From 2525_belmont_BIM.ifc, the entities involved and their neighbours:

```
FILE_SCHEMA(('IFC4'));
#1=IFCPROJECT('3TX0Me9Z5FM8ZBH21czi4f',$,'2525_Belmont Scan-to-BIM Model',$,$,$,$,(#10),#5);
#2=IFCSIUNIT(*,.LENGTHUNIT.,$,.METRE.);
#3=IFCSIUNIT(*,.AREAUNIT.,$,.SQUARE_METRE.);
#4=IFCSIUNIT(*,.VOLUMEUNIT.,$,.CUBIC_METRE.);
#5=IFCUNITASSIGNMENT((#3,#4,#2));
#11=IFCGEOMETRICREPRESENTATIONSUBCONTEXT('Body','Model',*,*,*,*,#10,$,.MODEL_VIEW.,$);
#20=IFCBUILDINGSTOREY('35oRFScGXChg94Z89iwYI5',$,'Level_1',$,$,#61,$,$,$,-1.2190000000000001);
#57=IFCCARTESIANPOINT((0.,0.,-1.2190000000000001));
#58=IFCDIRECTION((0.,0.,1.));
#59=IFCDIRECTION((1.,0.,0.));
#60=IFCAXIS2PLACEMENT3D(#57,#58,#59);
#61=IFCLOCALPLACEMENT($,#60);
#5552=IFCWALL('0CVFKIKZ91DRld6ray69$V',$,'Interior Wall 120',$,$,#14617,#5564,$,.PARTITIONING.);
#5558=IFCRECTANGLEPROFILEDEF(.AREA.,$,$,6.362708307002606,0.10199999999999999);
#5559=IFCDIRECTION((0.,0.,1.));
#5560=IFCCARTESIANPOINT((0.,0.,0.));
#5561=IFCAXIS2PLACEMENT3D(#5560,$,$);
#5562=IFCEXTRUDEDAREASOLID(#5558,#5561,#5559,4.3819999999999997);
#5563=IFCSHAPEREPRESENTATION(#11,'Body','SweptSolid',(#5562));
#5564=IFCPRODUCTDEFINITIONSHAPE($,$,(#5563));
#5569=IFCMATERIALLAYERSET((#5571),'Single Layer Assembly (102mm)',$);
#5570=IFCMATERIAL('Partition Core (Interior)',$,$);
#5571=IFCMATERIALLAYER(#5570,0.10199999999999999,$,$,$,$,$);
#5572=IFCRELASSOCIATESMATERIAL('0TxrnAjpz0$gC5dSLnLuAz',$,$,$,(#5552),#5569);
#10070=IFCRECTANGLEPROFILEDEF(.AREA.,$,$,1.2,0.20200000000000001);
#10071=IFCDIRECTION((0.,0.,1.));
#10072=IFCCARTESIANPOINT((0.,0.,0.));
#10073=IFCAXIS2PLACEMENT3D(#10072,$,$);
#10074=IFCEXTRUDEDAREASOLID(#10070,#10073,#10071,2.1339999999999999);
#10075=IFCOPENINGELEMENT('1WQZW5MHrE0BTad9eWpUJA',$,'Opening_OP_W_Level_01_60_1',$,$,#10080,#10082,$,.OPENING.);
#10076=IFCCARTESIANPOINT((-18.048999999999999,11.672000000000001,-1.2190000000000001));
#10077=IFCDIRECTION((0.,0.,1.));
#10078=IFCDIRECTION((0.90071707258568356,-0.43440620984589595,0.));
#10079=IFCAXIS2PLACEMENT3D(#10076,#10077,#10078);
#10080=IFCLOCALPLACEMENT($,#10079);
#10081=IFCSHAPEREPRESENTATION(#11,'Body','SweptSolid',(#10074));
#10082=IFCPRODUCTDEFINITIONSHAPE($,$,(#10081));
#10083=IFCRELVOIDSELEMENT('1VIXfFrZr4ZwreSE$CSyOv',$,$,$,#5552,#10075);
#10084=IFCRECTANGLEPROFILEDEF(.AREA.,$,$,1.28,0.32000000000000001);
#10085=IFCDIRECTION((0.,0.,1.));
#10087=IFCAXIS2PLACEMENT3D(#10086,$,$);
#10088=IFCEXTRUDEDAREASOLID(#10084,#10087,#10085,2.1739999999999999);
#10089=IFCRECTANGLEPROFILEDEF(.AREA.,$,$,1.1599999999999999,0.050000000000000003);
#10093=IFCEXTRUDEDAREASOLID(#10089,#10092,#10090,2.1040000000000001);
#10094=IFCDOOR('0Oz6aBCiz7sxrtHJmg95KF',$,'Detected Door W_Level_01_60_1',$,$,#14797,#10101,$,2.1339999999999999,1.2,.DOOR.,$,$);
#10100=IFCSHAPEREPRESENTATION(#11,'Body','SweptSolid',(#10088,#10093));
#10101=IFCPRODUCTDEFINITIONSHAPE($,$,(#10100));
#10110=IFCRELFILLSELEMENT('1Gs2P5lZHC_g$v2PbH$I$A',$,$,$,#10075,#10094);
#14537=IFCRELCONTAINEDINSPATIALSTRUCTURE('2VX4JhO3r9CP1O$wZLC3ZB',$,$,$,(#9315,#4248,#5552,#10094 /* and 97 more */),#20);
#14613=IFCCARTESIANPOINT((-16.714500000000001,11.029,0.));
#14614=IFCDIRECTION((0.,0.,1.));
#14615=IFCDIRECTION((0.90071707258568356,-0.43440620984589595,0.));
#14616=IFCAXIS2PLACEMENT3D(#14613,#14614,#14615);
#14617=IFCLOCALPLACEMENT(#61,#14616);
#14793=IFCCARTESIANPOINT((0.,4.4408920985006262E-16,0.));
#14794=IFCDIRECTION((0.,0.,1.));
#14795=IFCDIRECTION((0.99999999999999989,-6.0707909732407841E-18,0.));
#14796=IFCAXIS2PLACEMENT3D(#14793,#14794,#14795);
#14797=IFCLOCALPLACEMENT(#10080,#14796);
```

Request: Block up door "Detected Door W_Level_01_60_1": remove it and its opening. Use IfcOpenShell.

```python
import ifcopenshell
import ifcopenshell.api.feature
import ifcopenshell.api.root
import ifcopenshell.geom
import ifcopenshell.util.shape

model = ifcopenshell.open("2525_belmont_BIM.ifc")
settings = ifcopenshell.geom.settings()


def volume(element):
    """Net volume in cubic metres, openings subtracted."""
    shape = ifcopenshell.geom.create_shape(settings, element)
    return ifcopenshell.util.shape.get_volume(shape.geometry)


door = model.by_guid("0Oz6aBCiz7sxrtHJmg95KF")
opening = door.FillsVoids[0].RelatingOpeningElement
wall = opening.VoidsElements[0].RelatingBuildingElement
before = volume(wall)

ifcopenshell.api.root.remove_product(model, product=door)
ifcopenshell.api.feature.remove_feature(model, feature=opening)

after = volume(wall)

print(f"wall volume {before:.3f} -> {after:.3f} m3")

model.write("2525_belmont_BIM_updated.ifc")
```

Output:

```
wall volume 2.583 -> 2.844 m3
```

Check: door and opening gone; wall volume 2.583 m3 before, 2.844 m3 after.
